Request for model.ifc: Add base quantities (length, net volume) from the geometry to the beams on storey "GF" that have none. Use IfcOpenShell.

First a look at what the model holds.

```python
import ifcopenshell
import ifcopenshell.util.element
import ifcopenshell.util.unit

model = ifcopenshell.open("model.ifc")
print(model.schema)
for unit_type in ("LENGTHUNIT", "AREAUNIT", "VOLUMEUNIT"):
    print(unit_type, ifcopenshell.util.unit.calculate_unit_scale(model, unit_type))
storey = next(s for s in model.by_type("IfcBuildingStorey") if s.Name == "GF")
beams = [e for e in ifcopenshell.util.element.get_decomposition(storey) if e.is_a("IfcBeam")]
for e in sorted(beams, key=lambda e: e.id()):
    print(e.id(), e.is_a(), e.Name, list(ifcopenshell.util.element.get_psets(e, qtos_only=True)), sep=" | ")
```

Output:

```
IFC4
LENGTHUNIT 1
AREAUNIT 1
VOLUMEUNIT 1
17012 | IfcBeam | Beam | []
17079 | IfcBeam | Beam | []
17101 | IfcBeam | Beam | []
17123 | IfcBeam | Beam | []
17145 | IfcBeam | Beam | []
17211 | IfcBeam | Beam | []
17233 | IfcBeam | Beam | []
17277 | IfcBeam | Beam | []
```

```python
import ifcopenshell
import ifcopenshell.api.pset
import ifcopenshell.geom
import ifcopenshell.util.element
import ifcopenshell.util.shape
import ifcopenshell.util.unit

model = ifcopenshell.open("model.ifc")
unit_scale = ifcopenshell.util.unit.calculate_unit_scale(model)
volume_scale = ifcopenshell.util.unit.calculate_unit_scale(model, "VOLUMEUNIT")
settings = ifcopenshell.geom.settings()

storey = next(s for s in model.by_type("IfcBuildingStorey") if s.Name == "GF")
beams = [e for e in ifcopenshell.util.element.get_decomposition(storey) if e.is_a("IfcBeam")]

for e in sorted(beams, key=lambda e: e.id()):
    if ifcopenshell.util.element.get_psets(e, qtos_only=True, should_inherit=False):
        continue
    # Geometry comes back in metres, in the element's own axes.
    shape = ifcopenshell.geom.create_shape(settings, e)
    values = {
        "Length": ifcopenshell.util.shape.get_max_xyz(shape.geometry) / unit_scale,
        "NetVolume": ifcopenshell.util.shape.get_volume(shape.geometry) / volume_scale,
    }
    qto = ifcopenshell.api.pset.add_qto(model, product=e, name="Qto_BeamBaseQuantities")
    ifcopenshell.api.pset.edit_qto(model, qto=qto, properties=values)
    print(e.id(), {k: round(v, 3) for k, v in values.items()})

model.write("model-out.ifc")
```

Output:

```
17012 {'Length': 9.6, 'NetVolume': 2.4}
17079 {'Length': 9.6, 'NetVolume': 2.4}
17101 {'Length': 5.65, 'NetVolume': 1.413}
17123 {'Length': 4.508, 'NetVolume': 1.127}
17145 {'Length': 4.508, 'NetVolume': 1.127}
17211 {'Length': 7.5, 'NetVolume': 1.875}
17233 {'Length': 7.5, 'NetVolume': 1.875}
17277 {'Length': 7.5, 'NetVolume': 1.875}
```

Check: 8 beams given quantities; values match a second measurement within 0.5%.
